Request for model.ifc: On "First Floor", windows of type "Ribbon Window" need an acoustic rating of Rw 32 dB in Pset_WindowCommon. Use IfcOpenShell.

First a look at what the model holds.

```python
import ifcopenshell
import ifcopenshell.util.element

model = ifcopenshell.open("model.ifc")
print(model.schema)
storey = next(s for s in model.by_type("IfcBuildingStorey") if s.Name == "First Floor")
windows = [e for e in ifcopenshell.util.element.get_decomposition(storey) if e.is_a("IfcWindow")]
seen = {}
for e in windows:
    element_type = ifcopenshell.util.element.get_type(e)
    key = (element_type.Name if element_type != e and element_type else None, ifcopenshell.util.element.get_pset(e, "Pset_WindowCommon", "AcousticRating"))
    seen[key] = seen.get(key, 0) + 1
for (name, value), count in sorted(seen.items(), key=str):
    print(count, "x", name, "|", value)
```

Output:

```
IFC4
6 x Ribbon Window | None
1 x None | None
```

```python
import ifcopenshell
import ifcopenshell.api.pset
import ifcopenshell.util.element

model = ifcopenshell.open("model.ifc")

storey = next(s for s in model.by_type("IfcBuildingStorey") if s.Name == "First Floor")
windows = [e for e in ifcopenshell.util.element.get_decomposition(storey) if e.is_a("IfcWindow")]

count = 0
for e in windows:
    element_type = ifcopenshell.util.element.get_type(e)
    if element_type in (None, e) or element_type.Name != "Ribbon Window":
        continue
    # add_pset returns the element's existing set when there is one.
    pset = ifcopenshell.api.pset.add_pset(model, product=e, name="Pset_WindowCommon")
    ifcopenshell.api.pset.edit_pset(model, pset=pset, properties={"AcousticRating": "Rw 32 dB"})
    count += 1

print(count, "windows updated")

model.write("model_v2.ifc")
```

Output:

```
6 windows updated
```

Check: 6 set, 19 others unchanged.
